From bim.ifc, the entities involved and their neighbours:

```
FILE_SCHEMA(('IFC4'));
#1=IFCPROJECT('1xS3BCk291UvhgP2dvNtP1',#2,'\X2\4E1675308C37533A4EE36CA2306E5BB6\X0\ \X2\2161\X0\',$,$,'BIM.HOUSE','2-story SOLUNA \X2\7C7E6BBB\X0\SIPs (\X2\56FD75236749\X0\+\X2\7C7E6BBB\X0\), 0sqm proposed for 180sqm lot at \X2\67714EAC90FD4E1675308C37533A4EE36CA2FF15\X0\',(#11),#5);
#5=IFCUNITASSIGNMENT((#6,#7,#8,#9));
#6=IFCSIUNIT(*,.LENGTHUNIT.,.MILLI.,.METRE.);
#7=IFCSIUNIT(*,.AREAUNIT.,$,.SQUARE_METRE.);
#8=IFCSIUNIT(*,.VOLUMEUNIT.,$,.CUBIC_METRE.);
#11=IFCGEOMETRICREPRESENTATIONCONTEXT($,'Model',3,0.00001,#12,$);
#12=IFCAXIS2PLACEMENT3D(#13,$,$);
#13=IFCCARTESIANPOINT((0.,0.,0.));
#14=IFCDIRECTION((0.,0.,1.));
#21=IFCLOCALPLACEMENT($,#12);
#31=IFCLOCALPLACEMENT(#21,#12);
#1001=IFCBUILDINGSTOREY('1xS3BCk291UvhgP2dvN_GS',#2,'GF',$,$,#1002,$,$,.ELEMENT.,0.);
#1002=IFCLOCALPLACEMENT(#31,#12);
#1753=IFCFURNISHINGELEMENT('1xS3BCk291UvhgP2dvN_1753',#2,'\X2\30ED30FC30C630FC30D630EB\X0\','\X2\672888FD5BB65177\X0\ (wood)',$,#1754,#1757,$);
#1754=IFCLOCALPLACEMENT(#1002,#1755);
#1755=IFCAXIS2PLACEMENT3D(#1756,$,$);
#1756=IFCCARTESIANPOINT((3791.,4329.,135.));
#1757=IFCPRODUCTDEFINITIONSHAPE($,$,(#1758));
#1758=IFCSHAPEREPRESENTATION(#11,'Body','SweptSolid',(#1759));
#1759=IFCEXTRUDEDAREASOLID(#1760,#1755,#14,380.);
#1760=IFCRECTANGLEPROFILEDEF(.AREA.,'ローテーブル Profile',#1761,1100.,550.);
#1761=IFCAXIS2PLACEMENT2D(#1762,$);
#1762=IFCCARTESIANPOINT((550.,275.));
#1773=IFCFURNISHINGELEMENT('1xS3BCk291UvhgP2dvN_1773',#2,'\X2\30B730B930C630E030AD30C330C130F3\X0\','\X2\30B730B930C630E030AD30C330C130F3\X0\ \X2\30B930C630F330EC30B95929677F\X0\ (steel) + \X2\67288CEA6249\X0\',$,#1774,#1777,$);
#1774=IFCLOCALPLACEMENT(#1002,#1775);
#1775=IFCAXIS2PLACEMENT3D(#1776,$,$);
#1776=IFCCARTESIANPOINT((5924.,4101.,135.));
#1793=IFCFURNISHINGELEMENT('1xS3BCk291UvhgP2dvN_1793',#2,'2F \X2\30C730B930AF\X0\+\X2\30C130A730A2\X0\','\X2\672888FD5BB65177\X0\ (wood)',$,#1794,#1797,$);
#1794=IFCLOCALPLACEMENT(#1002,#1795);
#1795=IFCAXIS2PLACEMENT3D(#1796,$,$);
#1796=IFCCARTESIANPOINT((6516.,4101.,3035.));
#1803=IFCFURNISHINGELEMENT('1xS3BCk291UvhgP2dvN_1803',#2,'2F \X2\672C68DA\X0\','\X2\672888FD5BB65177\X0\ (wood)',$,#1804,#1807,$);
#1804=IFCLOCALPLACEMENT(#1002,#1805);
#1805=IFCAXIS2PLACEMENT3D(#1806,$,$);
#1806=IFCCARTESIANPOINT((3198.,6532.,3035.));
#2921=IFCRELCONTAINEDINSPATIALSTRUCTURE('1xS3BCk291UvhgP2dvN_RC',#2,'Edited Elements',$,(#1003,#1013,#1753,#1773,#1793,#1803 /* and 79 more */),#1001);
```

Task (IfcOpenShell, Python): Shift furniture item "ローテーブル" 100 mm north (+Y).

```python
import ifcopenshell
import ifcopenshell.api.geometry
import ifcopenshell.util.placement

model = ifcopenshell.open("bim.ifc")

item = model.by_guid("1xS3BCk291UvhgP2dvN_1753")
matrix = ifcopenshell.util.placement.get_local_placement(item.ObjectPlacement)
matrix[1, 3] += 100.0
ifcopenshell.api.geometry.edit_object_placement(model, product=item, matrix=matrix, is_si=False)

print(ifcopenshell.util.placement.get_local_placement(item.ObjectPlacement).round(3) + 0.0)

model.write("bim_v2.ifc")
```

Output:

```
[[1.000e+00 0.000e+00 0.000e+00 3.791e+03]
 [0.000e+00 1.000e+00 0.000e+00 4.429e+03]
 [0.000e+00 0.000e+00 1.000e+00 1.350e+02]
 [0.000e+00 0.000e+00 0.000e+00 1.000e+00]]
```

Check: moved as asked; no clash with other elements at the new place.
